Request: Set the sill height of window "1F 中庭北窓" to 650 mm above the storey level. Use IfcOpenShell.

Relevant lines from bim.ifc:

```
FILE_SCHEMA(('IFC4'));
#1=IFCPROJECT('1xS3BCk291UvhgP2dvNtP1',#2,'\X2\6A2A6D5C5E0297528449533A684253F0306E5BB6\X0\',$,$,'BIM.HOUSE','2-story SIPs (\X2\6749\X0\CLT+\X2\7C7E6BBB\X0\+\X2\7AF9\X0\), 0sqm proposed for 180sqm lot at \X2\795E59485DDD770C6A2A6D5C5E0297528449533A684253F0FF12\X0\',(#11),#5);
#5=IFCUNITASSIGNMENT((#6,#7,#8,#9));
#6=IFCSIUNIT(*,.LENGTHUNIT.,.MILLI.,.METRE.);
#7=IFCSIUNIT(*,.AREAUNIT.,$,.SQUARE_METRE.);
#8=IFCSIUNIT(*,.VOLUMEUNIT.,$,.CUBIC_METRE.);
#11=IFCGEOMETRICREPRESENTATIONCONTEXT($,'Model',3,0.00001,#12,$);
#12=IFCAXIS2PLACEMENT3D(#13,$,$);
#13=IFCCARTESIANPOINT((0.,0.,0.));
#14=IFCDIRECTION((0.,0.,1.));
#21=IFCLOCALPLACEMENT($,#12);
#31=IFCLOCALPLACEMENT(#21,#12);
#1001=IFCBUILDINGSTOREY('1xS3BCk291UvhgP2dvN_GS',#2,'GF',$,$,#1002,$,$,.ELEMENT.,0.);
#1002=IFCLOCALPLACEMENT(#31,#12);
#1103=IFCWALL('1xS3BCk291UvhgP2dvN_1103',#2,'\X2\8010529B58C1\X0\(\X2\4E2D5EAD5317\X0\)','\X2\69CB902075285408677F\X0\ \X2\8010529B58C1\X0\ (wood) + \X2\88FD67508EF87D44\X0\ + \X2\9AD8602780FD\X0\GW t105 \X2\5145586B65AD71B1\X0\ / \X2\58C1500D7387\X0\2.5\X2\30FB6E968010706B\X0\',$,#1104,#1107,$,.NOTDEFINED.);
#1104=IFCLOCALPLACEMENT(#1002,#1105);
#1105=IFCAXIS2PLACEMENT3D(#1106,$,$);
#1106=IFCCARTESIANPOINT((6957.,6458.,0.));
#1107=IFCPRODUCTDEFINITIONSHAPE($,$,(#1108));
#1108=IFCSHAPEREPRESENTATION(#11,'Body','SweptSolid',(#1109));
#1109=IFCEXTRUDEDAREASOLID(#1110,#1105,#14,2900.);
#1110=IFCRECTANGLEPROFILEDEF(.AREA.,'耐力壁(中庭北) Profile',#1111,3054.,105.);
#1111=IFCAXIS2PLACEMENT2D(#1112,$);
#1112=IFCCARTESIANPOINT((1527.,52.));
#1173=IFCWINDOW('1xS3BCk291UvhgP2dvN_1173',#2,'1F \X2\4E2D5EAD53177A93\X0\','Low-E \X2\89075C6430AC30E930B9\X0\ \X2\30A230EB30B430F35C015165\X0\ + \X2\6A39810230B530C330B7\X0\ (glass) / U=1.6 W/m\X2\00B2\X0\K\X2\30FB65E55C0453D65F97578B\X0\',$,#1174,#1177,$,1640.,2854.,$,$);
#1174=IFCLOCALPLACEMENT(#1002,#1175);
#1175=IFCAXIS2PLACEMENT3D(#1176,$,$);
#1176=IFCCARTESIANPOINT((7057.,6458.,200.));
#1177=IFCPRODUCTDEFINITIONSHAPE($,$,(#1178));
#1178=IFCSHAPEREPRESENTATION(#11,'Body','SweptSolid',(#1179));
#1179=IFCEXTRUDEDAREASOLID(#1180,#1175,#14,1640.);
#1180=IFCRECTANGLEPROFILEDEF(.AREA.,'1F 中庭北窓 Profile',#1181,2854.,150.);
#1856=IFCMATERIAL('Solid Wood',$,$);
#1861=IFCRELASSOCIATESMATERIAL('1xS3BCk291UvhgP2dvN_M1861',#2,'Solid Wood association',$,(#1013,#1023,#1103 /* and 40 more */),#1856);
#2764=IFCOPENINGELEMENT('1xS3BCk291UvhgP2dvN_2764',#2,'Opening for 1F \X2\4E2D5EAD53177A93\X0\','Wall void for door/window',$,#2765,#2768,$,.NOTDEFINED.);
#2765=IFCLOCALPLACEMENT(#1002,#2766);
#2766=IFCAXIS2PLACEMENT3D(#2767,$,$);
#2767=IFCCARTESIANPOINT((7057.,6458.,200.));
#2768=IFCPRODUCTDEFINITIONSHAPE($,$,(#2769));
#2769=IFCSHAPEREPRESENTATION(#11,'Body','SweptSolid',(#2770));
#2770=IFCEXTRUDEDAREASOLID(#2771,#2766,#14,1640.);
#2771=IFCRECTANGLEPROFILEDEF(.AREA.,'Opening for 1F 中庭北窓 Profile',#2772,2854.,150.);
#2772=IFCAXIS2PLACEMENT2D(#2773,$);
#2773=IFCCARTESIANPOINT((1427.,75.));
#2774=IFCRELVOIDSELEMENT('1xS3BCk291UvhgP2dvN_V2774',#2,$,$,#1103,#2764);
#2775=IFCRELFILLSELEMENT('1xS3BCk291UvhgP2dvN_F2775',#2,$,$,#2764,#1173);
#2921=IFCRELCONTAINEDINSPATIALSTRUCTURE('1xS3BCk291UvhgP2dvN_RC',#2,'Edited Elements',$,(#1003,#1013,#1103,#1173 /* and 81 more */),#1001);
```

```python
import numpy as np
import ifcopenshell
import ifcopenshell.api.geometry
import ifcopenshell.geom
import ifcopenshell.util.element
import ifcopenshell.util.placement
import ifcopenshell.util.shape
import ifcopenshell.util.unit

model = ifcopenshell.open("bim.ifc")
unit_scale = ifcopenshell.util.unit.calculate_unit_scale(model)

window = model.by_guid("1xS3BCk291UvhgP2dvN_1173")
opening = window.FillsVoids[0].RelatingOpeningElement
storey = ifcopenshell.util.element.get_container(window, ifc_class="IfcBuildingStorey")
level = ifcopenshell.util.placement.get_local_placement(storey.ObjectPlacement)[2, 3]

# The opening's origin need not be at the sill, so measure its lowest point.
shape = ifcopenshell.geom.create_shape(ifcopenshell.geom.settings(), opening)
bottom = ifcopenshell.util.shape.get_shape_bottom_elevation(shape, shape.geometry) / unit_scale
dz = level + 650.0 - bottom

shift = np.array([0.0, 0.0, dz])
# The window is not placed relative to its opening, so move both.
for product in (opening, window):
    matrix = ifcopenshell.util.placement.get_local_placement(product.ObjectPlacement)
    matrix[:3, 3] += shift
    ifcopenshell.api.geometry.edit_object_placement(model, product=product, matrix=matrix, is_si=False)

print(f"moved by {dz * unit_scale:+.3f} m")

model.write("bim_updated.ifc")
```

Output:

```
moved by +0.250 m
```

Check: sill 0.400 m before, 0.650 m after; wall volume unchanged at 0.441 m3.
